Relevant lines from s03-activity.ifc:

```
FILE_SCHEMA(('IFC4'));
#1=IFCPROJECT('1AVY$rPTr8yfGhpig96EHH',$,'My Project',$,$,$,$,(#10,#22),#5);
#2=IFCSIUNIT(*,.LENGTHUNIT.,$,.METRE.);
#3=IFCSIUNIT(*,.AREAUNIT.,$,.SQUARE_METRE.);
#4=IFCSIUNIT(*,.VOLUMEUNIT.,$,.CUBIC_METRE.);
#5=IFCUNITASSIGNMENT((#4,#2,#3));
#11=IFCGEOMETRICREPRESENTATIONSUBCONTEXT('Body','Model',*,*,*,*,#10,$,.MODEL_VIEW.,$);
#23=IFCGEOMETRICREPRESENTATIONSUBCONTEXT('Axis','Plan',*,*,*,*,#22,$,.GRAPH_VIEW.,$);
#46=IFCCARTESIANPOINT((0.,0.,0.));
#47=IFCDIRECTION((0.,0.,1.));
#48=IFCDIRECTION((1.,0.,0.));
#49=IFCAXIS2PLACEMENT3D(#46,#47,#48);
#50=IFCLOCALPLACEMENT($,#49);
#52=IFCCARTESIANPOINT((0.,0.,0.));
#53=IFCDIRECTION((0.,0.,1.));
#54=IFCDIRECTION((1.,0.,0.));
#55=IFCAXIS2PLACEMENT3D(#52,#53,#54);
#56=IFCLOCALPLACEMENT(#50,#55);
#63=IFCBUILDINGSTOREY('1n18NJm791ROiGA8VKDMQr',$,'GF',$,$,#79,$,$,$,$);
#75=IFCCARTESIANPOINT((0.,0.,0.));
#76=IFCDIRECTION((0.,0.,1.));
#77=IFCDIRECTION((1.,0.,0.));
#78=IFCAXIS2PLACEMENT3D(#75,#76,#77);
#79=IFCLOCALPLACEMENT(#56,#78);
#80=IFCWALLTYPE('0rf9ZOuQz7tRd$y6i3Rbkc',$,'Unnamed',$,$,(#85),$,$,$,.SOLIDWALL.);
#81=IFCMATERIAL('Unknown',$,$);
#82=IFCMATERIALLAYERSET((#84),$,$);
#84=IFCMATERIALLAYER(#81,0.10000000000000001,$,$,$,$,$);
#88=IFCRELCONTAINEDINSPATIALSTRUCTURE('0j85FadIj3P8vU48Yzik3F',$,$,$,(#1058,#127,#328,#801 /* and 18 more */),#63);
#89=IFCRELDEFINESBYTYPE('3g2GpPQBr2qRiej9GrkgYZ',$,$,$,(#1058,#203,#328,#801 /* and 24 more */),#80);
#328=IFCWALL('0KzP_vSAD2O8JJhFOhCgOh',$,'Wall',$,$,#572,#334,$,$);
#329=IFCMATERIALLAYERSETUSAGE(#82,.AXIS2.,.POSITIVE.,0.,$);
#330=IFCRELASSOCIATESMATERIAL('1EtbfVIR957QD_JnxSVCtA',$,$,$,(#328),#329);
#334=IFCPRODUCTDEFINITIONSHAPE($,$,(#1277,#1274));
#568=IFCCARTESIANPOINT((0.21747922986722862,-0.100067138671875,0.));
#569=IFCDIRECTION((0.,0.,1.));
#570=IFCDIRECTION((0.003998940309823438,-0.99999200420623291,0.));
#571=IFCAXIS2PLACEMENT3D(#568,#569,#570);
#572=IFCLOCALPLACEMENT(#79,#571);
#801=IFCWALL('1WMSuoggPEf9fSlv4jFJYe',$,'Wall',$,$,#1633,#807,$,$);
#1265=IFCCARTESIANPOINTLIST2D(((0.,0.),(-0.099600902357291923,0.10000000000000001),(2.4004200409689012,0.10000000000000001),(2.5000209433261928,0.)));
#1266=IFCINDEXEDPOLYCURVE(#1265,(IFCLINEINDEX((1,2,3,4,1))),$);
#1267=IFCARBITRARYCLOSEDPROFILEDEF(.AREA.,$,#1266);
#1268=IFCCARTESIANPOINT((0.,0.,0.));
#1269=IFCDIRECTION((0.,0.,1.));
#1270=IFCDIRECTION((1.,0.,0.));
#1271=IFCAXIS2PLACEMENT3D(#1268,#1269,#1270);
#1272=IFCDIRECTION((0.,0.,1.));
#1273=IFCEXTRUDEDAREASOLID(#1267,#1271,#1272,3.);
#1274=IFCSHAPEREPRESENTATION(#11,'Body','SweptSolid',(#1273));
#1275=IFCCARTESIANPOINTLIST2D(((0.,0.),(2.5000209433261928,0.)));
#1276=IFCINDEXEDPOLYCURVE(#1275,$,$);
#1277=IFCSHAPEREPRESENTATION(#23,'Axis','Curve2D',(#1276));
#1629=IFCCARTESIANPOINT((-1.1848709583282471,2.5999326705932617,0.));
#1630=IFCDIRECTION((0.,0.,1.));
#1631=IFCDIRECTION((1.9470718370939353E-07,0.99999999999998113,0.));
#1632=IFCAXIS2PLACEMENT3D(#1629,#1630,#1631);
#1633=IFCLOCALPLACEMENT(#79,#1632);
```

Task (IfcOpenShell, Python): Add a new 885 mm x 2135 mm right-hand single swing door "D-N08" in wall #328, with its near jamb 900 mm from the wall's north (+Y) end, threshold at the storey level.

```python
import numpy as np
import ifcopenshell
import ifcopenshell.api.feature
import ifcopenshell.api.geometry
import ifcopenshell.api.root
import ifcopenshell.api.spatial
import ifcopenshell.geom
import ifcopenshell.util.element
import ifcopenshell.util.placement
import ifcopenshell.util.representation
import ifcopenshell.util.shape
import ifcopenshell.util.unit

model = ifcopenshell.open("s03-activity.ifc")
unit_scale = ifcopenshell.util.unit.calculate_unit_scale(model)
settings = ifcopenshell.geom.settings()


def volume(element):
    """Net volume in cubic metres, openings subtracted."""
    shape = ifcopenshell.geom.create_shape(settings, element)
    return ifcopenshell.util.shape.get_volume(shape.geometry)


wall = model.by_guid("0KzP_vSAD2O8JJhFOhCgOh")
storey = ifcopenshell.util.element.get_container(wall, ifc_class="IfcBuildingStorey")
context = ifcopenshell.util.representation.get_context(model, "Model", "Body", "MODEL_VIEW")
before = volume(wall)

width, height, from_end, sill = 0.885, 2.135, 0.9, 0.0  # metres

# The wall runs along its own X axis, and the end named is its -X end.
wall_shape = ifcopenshell.geom.create_shape(settings, wall)
x, y, z = ifcopenshell.util.shape.get_vertices(wall_shape.geometry).T
start = x.min() + from_end
face, thickness = float(y.min()), float(y.max() - y.min())
wall_matrix = ifcopenshell.util.placement.get_local_placement(wall.ObjectPlacement)
level = ifcopenshell.util.placement.get_local_placement(storey.ObjectPlacement)[2, 3]


def in_wall(x, y):
    """Placement at x, y metres in the wall's axes, at sill height."""
    matrix = wall_matrix.copy()
    matrix[:, 3] = wall_matrix @ np.array([x / unit_scale, y / unit_scale, 0.0, 1.0])
    matrix[2, 3] = level + sill / unit_scale
    return matrix


# Opening: a box that overshoots both wall faces by 50 mm.
opening = ifcopenshell.api.root.create_entity(model, ifc_class="IfcOpeningElement", predefined_type="OPENING")
box = ifcopenshell.api.geometry.add_wall_representation(
    model, context=context, length=width, height=height, thickness=thickness + 0.1
)
ifcopenshell.api.geometry.assign_representation(model, product=opening, representation=box)
ifcopenshell.api.geometry.edit_object_placement(model, product=opening, matrix=in_wall(start, face - 0.05), is_si=False)
ifcopenshell.api.feature.add_feature(model, feature=opening, element=wall)

door = ifcopenshell.api.root.create_entity(model, ifc_class="IfcDoor", name="D-N08", predefined_type="DOOR")
door.OverallWidth, door.OverallHeight = width / unit_scale, height / unit_scale
door.OperationType = "SINGLE_SWING_RIGHT"
body = ifcopenshell.api.geometry.add_door_representation(
    model,
    context=context,
    overall_width=door.OverallWidth,
    overall_height=door.OverallHeight,
    operation_type="SINGLE_SWING_RIGHT",
    lining_properties={"LiningDepth": thickness / unit_scale, "ThresholdDepth": thickness / unit_scale},
)
ifcopenshell.api.geometry.assign_representation(model, product=door, representation=body)
ifcopenshell.api.spatial.assign_container(model, products=[door], relating_structure=storey)
ifcopenshell.api.feature.add_filling(model, opening=opening, element=door)

# The lining spans the wall, so the door starts at the wall face.
ifcopenshell.api.geometry.edit_object_placement(model, product=door, matrix=in_wall(start, face), is_si=False)

after = volume(wall)

print(f"wall volume {before:.3f} -> {after:.3f} m3")

model.write("s03-activity_v2.ifc")
```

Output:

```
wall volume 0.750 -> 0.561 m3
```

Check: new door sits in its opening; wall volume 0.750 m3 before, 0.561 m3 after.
